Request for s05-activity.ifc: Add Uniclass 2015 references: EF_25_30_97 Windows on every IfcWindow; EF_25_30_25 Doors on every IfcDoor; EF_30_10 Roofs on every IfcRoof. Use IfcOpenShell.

First a look at what the model holds.

```python
import ifcopenshell

model = ifcopenshell.open("s05-activity.ifc")
print(model.schema)
print("classifications:", [c.Name for c in model.by_type("IfcClassification")])
for ifc_class in ("IfcDoor", "IfcRoof", "IfcStair", "IfcWall", "IfcWindow"):
    print(ifc_class, len(model.by_type(ifc_class)))
```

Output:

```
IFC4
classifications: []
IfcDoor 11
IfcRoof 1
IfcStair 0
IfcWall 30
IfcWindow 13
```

```python
import ifcopenshell
import ifcopenshell.api.classification

model = ifcopenshell.open("s05-activity.ifc")

system = ifcopenshell.api.classification.add_classification(model, classification="Uniclass 2015")

codes = {
    "IfcWindow": ("EF_25_30_97", "Windows"),
    "IfcDoor": ("EF_25_30_25", "Doors"),
    "IfcRoof": ("EF_30_10", "Roofs"),
}
for ifc_class, (code, name) in codes.items():
    products = model.by_type(ifc_class)
    ifcopenshell.api.classification.add_reference(
        model, products=products, classification=system, identification=code, name=name
    )
    print(code, len(products))

model.write("s05-activity-out.ifc")
```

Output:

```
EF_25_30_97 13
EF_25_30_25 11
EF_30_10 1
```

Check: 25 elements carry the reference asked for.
